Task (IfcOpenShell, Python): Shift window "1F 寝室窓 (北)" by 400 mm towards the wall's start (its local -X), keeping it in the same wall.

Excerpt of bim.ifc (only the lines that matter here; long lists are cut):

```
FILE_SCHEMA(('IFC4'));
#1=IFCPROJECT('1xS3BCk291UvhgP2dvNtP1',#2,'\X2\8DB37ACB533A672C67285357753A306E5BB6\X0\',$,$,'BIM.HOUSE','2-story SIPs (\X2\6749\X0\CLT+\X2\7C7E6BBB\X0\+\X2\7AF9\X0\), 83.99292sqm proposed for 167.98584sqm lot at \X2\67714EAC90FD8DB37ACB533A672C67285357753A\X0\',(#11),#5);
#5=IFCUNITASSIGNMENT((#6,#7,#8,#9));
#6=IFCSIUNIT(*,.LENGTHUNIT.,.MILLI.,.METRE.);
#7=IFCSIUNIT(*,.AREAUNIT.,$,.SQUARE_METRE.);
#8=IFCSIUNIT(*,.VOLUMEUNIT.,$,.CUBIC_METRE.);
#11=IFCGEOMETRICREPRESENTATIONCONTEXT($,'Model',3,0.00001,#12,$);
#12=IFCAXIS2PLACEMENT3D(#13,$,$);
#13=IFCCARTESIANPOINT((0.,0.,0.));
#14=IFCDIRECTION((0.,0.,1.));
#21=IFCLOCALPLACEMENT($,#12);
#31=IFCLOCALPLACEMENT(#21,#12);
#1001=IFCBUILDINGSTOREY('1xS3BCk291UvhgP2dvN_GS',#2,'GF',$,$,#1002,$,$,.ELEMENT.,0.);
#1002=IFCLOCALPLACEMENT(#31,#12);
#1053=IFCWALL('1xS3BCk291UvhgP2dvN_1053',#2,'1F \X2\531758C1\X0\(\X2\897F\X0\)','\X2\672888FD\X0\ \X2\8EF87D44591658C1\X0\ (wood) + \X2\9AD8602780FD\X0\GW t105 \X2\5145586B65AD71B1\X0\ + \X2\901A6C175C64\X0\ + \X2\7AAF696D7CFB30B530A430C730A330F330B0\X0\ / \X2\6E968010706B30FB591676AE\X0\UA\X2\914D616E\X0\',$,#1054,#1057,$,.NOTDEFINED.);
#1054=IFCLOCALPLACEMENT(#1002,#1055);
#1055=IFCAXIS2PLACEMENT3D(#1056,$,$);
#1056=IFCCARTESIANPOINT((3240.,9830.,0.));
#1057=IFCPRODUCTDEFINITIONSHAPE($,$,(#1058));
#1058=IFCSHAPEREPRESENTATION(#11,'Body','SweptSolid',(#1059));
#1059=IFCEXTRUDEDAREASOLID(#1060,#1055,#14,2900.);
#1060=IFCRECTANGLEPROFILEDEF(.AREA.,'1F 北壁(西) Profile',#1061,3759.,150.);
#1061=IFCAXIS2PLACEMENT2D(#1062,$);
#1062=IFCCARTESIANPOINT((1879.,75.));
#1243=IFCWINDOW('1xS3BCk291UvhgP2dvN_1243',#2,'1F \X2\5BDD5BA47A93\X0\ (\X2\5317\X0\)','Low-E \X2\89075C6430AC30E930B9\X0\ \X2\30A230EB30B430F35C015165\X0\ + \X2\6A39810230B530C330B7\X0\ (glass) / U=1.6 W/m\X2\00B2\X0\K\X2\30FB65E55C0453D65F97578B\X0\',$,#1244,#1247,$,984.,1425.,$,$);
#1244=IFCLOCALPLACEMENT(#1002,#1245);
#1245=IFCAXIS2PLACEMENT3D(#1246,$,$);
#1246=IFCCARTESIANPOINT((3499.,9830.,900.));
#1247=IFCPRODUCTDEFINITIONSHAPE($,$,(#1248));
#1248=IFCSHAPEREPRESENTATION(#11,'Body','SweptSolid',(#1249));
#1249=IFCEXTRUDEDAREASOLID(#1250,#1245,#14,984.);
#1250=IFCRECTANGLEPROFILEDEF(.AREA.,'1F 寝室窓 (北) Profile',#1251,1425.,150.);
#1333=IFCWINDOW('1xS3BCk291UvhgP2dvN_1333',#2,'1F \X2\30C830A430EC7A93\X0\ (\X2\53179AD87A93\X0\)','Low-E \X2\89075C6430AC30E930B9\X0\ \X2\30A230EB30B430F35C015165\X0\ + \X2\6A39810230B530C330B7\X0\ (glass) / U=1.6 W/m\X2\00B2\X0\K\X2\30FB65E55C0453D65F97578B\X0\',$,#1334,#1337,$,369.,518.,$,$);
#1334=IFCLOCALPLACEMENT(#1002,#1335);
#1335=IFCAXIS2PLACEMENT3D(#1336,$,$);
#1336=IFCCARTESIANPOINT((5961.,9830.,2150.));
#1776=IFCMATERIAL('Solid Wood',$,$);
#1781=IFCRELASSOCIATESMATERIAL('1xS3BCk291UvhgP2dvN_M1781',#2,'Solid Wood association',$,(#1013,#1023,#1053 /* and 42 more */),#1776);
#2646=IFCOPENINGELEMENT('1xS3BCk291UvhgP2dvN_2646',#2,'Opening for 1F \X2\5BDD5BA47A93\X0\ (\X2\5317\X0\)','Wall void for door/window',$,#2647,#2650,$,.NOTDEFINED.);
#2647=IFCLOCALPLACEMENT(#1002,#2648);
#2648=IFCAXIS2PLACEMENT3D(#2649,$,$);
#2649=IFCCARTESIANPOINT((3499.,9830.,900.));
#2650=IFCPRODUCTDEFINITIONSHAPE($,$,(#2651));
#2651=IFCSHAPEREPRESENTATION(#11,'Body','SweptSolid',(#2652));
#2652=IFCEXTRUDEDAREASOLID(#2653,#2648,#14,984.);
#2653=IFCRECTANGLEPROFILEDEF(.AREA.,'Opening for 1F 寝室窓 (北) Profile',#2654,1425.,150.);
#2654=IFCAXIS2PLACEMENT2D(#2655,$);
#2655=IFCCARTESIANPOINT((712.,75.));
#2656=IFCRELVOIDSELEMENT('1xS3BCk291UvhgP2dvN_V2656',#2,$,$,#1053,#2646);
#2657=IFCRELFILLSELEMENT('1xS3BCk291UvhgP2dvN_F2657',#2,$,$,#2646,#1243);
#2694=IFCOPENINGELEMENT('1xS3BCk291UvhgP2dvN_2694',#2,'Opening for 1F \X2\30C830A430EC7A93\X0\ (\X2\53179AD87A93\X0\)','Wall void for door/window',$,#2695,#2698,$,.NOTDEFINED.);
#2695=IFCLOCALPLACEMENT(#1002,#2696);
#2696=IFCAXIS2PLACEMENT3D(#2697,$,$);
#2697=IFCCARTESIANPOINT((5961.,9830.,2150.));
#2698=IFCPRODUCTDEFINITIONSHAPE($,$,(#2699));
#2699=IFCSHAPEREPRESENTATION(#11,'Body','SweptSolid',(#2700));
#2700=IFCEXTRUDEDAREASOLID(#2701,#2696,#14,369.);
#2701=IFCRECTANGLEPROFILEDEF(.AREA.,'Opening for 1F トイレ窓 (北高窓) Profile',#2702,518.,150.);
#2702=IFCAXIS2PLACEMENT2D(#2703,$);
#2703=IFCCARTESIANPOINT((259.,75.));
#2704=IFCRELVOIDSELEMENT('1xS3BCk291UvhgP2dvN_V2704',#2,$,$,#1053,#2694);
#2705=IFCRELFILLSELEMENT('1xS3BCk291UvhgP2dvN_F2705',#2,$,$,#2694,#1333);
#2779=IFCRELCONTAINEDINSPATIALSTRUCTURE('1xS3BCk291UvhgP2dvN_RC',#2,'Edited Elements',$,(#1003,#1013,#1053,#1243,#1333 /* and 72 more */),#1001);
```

```python
import ifcopenshell
import ifcopenshell.api.geometry
import ifcopenshell.util.placement

model = ifcopenshell.open("bim.ifc")

window = model.by_guid("1xS3BCk291UvhgP2dvN_1243")
opening = window.FillsVoids[0].RelatingOpeningElement
wall = opening.VoidsElements[0].RelatingBuildingElement

wall_matrix = ifcopenshell.util.placement.get_local_placement(wall.ObjectPlacement)
shift = wall_matrix[:3, 0] * -400.0
before = ifcopenshell.util.placement.get_local_placement(window.ObjectPlacement)[:3, 3].copy()

# The window is not placed relative to its opening, so move both.
for product in (opening, window):
    matrix = ifcopenshell.util.placement.get_local_placement(product.ObjectPlacement)
    matrix[:3, 3] += shift
    ifcopenshell.api.geometry.edit_object_placement(model, product=product, matrix=matrix, is_si=False)

after = ifcopenshell.util.placement.get_local_placement(window.ObjectPlacement)[:3, 3]
print("window moved by", (after - before).round(3) + 0.0)

model.write("bim_rev.ifc")
```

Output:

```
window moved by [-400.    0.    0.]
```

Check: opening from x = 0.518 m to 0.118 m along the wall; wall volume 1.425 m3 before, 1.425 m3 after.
